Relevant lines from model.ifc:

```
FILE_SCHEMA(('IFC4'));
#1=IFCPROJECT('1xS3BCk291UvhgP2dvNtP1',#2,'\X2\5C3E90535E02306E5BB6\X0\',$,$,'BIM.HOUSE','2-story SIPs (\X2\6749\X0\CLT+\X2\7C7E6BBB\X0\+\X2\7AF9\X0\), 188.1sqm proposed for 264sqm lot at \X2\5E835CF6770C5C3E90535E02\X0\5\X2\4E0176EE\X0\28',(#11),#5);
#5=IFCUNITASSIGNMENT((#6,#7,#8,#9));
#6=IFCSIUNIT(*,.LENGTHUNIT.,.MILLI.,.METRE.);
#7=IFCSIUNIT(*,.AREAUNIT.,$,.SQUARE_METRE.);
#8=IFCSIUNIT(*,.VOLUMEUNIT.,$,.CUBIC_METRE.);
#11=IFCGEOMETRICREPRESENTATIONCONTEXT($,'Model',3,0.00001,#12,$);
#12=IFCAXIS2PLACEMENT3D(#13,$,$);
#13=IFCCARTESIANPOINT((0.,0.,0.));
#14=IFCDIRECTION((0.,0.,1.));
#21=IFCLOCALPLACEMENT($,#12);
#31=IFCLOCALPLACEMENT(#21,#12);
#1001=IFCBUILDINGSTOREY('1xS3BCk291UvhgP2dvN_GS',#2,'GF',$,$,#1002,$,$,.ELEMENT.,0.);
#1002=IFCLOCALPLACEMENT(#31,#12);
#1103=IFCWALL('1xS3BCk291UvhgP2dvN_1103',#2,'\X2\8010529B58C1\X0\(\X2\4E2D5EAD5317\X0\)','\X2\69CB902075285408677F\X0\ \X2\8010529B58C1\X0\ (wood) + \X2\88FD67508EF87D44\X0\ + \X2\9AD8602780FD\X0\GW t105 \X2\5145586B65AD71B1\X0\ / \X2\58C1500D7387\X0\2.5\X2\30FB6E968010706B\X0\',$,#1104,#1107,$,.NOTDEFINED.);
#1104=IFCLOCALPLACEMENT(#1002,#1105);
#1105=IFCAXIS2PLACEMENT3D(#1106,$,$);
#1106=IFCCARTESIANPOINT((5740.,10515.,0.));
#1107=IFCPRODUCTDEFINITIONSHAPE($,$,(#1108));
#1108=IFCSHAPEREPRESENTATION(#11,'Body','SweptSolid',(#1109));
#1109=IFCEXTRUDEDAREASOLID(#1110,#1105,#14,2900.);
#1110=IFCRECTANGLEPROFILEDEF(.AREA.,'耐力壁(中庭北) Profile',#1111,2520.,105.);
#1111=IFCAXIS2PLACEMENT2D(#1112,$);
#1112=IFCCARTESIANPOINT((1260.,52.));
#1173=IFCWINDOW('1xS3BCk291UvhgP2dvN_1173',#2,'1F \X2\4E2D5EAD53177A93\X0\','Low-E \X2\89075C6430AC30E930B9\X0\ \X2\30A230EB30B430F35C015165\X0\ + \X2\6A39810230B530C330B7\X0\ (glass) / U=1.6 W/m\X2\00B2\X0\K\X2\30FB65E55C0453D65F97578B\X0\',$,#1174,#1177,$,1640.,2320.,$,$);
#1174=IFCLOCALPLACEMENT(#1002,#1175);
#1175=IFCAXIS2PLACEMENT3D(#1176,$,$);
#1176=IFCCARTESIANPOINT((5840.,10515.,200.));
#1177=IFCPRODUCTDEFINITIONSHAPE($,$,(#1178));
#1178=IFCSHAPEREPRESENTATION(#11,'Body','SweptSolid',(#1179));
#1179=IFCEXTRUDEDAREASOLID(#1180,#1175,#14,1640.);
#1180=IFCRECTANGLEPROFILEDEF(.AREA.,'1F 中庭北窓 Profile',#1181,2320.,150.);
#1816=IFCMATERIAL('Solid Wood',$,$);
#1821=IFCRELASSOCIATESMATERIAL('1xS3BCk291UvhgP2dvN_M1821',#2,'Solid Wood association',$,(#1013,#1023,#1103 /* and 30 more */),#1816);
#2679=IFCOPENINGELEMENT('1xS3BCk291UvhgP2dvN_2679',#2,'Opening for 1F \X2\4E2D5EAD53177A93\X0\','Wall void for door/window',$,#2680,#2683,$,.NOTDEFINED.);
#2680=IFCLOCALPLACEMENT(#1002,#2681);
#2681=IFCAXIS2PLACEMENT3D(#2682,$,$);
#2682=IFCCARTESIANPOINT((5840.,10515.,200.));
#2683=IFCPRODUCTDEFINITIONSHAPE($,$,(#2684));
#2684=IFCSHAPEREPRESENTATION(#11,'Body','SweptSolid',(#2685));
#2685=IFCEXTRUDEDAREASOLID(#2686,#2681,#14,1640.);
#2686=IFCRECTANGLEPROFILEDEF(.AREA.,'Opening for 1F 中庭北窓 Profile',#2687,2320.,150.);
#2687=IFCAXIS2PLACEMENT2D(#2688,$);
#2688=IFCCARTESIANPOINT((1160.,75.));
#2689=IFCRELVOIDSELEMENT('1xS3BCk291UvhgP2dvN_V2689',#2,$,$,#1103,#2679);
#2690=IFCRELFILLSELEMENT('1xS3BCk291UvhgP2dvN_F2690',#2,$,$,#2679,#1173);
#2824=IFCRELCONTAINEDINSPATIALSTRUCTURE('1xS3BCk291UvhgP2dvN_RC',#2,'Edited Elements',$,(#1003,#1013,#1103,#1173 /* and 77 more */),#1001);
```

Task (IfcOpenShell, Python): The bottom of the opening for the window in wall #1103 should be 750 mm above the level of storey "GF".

```python
import numpy as np
import ifcopenshell
import ifcopenshell.api.geometry
import ifcopenshell.geom
import ifcopenshell.util.element
import ifcopenshell.util.placement
import ifcopenshell.util.shape
import ifcopenshell.util.unit

model = ifcopenshell.open("model.ifc")
unit_scale = ifcopenshell.util.unit.calculate_unit_scale(model)

window = model.by_guid("1xS3BCk291UvhgP2dvN_1173")
opening = window.FillsVoids[0].RelatingOpeningElement
storey = ifcopenshell.util.element.get_container(window, ifc_class="IfcBuildingStorey")
level = ifcopenshell.util.placement.get_local_placement(storey.ObjectPlacement)[2, 3]

# The opening's origin need not be at the sill, so measure its lowest point.
shape = ifcopenshell.geom.create_shape(ifcopenshell.geom.settings(), opening)
bottom = ifcopenshell.util.shape.get_shape_bottom_elevation(shape, shape.geometry) / unit_scale
dz = level + 0.75 / unit_scale - bottom

shift = np.array([0.0, 0.0, dz])
# The window is not placed relative to its opening, so move both.
for product in (opening, window):
    matrix = ifcopenshell.util.placement.get_local_placement(product.ObjectPlacement)
    matrix[:3, 3] += shift
    ifcopenshell.api.geometry.edit_object_placement(model, product=product, matrix=matrix, is_si=False)

print(f"moved by {dz * unit_scale:+.3f} m")

model.write("model_v2.ifc")
```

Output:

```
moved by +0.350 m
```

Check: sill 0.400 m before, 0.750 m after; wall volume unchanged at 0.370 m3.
